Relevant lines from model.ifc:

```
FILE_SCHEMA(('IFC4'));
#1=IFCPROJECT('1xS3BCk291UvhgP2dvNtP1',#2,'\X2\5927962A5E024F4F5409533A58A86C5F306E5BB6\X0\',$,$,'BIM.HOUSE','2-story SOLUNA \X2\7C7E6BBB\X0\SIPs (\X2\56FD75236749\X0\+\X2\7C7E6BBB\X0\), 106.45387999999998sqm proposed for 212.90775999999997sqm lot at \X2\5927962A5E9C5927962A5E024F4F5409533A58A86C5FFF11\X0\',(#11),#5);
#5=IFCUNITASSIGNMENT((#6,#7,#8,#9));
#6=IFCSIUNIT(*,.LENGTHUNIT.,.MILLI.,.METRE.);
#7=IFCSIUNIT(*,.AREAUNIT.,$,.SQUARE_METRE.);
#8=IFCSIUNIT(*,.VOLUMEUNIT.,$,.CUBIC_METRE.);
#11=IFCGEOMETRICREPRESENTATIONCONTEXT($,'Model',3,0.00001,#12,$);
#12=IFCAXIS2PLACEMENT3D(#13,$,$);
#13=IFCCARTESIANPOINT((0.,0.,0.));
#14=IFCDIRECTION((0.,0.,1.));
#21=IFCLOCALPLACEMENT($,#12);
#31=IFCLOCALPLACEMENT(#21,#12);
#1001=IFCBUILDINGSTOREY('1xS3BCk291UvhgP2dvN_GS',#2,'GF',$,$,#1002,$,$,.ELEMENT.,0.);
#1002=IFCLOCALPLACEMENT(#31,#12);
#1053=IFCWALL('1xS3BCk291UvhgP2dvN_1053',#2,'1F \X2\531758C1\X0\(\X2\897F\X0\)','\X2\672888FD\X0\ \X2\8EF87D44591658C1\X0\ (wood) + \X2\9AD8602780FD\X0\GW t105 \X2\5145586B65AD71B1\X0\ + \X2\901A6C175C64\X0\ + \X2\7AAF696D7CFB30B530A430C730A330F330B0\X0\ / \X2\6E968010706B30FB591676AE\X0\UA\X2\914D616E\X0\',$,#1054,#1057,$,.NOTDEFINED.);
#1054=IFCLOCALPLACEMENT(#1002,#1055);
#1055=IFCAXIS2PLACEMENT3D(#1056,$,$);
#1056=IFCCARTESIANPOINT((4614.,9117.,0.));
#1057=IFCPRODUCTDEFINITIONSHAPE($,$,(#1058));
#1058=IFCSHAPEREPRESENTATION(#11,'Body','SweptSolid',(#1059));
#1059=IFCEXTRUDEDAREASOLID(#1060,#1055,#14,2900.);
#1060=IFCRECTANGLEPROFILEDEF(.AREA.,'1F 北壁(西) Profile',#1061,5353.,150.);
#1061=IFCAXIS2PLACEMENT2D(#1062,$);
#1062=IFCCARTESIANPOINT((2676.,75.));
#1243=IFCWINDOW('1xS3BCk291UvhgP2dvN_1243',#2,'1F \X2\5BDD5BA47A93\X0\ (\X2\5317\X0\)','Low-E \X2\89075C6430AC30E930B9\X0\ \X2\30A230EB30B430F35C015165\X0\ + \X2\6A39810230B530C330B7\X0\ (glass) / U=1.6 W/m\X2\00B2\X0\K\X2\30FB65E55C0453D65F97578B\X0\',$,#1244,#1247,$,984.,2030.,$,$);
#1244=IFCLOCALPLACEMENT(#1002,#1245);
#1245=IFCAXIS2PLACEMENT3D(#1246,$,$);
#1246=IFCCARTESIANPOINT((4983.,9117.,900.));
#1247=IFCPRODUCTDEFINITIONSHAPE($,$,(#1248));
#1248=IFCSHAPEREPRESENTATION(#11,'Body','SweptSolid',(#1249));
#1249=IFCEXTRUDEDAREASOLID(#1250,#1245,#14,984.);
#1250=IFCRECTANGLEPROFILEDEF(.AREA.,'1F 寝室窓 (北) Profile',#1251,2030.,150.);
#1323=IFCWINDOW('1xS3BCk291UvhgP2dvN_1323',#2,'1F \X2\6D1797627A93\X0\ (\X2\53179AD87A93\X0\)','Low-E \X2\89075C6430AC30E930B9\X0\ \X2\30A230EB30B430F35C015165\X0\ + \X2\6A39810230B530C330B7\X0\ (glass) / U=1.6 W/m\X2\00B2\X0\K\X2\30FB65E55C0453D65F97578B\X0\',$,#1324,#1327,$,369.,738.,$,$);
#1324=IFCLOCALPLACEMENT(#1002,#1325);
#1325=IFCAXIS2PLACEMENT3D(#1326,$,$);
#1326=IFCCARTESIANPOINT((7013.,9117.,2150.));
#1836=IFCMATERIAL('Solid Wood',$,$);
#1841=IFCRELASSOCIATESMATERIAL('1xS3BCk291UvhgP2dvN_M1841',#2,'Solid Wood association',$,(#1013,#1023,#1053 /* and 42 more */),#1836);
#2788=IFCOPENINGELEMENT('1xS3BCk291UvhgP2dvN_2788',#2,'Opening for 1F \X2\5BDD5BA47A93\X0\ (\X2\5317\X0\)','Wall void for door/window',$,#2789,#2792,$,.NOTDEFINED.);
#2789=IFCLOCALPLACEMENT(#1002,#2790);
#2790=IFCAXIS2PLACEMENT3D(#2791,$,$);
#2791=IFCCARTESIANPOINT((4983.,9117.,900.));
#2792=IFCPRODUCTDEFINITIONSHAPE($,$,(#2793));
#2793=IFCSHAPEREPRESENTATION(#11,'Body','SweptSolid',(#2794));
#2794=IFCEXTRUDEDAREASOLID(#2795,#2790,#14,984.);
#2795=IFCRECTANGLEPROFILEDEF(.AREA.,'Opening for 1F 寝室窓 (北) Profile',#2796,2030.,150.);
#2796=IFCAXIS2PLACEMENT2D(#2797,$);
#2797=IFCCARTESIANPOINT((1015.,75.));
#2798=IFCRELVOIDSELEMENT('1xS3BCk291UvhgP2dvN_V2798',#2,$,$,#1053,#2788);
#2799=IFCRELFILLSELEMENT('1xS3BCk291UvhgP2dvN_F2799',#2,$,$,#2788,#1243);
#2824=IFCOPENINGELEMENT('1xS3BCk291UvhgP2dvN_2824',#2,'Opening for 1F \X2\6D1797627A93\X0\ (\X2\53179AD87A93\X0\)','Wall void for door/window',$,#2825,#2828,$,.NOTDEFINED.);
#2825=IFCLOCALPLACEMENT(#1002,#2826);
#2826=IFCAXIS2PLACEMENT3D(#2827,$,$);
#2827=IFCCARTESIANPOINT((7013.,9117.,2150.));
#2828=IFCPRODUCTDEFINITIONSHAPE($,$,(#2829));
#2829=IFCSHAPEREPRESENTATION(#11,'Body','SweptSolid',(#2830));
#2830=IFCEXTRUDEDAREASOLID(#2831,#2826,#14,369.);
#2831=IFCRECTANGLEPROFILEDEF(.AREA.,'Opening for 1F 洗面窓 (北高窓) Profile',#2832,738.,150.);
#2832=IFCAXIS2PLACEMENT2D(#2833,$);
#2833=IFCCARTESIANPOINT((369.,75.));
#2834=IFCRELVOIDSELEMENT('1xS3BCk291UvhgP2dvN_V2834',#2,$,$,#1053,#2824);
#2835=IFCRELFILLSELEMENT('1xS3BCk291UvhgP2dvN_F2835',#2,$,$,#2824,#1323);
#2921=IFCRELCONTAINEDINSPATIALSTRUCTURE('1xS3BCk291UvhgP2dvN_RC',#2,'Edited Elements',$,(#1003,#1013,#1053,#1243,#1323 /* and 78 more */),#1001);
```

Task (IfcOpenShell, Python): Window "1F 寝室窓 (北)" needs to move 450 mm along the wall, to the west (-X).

```python
import ifcopenshell
import ifcopenshell.api.geometry
import ifcopenshell.util.placement
import ifcopenshell.util.unit

model = ifcopenshell.open("model.ifc")
unit_scale = ifcopenshell.util.unit.calculate_unit_scale(model)

window = model.by_guid("1xS3BCk291UvhgP2dvN_1243")
opening = window.FillsVoids[0].RelatingOpeningElement
wall = opening.VoidsElements[0].RelatingBuildingElement

wall_matrix = ifcopenshell.util.placement.get_local_placement(wall.ObjectPlacement)
shift = wall_matrix[:3, 0] * -0.45 / unit_scale
before = ifcopenshell.util.placement.get_local_placement(window.ObjectPlacement)[:3, 3].copy()

# The window is not placed relative to its opening, so move both.
for product in (opening, window):
    matrix = ifcopenshell.util.placement.get_local_placement(product.ObjectPlacement)
    matrix[:3, 3] += shift
    ifcopenshell.api.geometry.edit_object_placement(model, product=product, matrix=matrix, is_si=False)

after = ifcopenshell.util.placement.get_local_placement(window.ObjectPlacement)[:3, 3]
print("window moved by", (after - before).round(3) + 0.0)

model.write("model_updated.ifc")
```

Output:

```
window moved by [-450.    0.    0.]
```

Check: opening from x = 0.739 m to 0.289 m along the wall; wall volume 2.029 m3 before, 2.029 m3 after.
